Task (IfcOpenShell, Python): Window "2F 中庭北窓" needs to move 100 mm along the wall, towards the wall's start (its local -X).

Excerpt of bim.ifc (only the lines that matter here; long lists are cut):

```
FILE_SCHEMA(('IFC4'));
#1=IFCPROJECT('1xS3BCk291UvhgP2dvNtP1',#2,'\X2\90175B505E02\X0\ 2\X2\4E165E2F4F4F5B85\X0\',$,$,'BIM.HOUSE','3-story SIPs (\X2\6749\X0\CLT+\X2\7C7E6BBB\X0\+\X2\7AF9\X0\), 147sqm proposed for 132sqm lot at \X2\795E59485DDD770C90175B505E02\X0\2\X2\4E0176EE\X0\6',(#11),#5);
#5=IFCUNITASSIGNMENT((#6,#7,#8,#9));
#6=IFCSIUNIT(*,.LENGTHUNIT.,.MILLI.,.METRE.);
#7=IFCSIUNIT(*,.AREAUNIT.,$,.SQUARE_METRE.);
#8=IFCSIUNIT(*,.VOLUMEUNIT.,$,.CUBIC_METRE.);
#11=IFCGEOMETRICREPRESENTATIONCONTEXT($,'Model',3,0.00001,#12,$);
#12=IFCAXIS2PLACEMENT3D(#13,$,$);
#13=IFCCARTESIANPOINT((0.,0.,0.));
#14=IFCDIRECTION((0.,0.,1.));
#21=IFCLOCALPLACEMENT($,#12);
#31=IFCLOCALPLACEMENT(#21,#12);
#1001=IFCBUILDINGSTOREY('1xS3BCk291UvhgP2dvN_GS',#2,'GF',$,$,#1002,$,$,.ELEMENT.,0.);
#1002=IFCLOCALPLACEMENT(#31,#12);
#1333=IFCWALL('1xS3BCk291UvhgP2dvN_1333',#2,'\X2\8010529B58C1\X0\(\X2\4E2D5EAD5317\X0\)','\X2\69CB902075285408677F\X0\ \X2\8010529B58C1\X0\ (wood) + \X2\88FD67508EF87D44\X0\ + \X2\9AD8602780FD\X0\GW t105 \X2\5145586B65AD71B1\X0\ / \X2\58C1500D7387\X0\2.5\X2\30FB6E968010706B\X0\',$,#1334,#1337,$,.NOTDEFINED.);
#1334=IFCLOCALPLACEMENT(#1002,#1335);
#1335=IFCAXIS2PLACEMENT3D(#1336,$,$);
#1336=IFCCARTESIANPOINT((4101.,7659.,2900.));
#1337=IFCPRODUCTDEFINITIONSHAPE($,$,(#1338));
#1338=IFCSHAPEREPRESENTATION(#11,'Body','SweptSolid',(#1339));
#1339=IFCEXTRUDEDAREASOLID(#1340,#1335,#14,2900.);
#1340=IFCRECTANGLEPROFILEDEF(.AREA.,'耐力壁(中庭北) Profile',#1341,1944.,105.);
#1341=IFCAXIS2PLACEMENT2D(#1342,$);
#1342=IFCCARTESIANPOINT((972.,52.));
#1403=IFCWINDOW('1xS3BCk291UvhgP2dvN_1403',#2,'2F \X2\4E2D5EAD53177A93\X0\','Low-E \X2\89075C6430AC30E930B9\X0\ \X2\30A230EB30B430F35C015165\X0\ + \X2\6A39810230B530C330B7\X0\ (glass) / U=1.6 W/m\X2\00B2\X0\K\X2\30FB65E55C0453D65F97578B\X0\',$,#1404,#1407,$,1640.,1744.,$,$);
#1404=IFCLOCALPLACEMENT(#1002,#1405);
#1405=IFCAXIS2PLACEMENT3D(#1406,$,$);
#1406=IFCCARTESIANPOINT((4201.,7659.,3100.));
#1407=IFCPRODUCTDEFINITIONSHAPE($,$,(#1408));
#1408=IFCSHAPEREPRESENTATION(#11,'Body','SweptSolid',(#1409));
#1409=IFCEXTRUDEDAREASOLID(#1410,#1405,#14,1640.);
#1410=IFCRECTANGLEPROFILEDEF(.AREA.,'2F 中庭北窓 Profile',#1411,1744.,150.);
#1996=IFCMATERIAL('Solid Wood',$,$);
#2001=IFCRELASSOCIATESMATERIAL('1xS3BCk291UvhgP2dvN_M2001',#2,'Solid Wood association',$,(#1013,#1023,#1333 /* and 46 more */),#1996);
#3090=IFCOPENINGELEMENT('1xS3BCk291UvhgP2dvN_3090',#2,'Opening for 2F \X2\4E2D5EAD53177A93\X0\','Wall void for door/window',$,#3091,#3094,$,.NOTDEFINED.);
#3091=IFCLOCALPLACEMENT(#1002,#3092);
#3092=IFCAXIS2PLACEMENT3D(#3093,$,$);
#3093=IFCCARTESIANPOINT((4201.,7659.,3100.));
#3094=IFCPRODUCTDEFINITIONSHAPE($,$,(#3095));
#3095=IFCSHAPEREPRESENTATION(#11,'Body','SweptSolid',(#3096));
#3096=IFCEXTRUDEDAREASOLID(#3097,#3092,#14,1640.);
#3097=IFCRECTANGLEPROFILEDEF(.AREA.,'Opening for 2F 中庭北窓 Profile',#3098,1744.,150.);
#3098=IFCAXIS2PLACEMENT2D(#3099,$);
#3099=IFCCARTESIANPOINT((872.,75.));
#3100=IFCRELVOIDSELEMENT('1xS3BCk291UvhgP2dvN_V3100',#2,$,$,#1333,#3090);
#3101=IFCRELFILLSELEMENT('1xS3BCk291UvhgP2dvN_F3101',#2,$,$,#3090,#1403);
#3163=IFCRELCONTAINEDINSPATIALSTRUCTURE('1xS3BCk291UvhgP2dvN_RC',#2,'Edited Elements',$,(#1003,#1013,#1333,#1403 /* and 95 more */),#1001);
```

```python
import ifcopenshell
import ifcopenshell.api.geometry
import ifcopenshell.util.placement

model = ifcopenshell.open("bim.ifc")

window = model.by_guid("1xS3BCk291UvhgP2dvN_1403")
opening = window.FillsVoids[0].RelatingOpeningElement
wall = opening.VoidsElements[0].RelatingBuildingElement

wall_matrix = ifcopenshell.util.placement.get_local_placement(wall.ObjectPlacement)
shift = wall_matrix[:3, 0] * -100.0
before = ifcopenshell.util.placement.get_local_placement(window.ObjectPlacement)[:3, 3].copy()

# The window is not placed relative to its opening, so move both.
for product in (opening, window):
    matrix = ifcopenshell.util.placement.get_local_placement(product.ObjectPlacement)
    matrix[:3, 3] += shift
    ifcopenshell.api.geometry.edit_object_placement(model, product=product, matrix=matrix, is_si=False)

after = ifcopenshell.util.placement.get_local_placement(window.ObjectPlacement)[:3, 3]
print("window moved by", (after - before).round(3) + 0.0)

model.write("bim_updated.ifc")
```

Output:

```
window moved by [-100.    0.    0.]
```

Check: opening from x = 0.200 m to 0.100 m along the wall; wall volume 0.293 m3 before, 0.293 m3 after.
